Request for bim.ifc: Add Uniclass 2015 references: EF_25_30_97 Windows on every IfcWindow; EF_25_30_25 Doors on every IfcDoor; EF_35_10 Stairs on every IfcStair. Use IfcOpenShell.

First a look at what the model holds.

```python
import ifcopenshell

model = ifcopenshell.open("bim.ifc")
print(model.schema)
print("classifications:", [c.Name for c in model.by_type("IfcClassification")])
for ifc_class in ("IfcDoor", "IfcRoof", "IfcStair", "IfcWall", "IfcWindow"):
    print(ifc_class, len(model.by_type(ifc_class)))
```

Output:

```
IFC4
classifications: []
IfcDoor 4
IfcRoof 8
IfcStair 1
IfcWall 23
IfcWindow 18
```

```python
import ifcopenshell
import ifcopenshell.api.classification

model = ifcopenshell.open("bim.ifc")

system = ifcopenshell.api.classification.add_classification(model, classification="Uniclass 2015")

codes = {
    "IfcWindow": ("EF_25_30_97", "Windows"),
    "IfcDoor": ("EF_25_30_25", "Doors"),
    "IfcStair": ("EF_35_10", "Stairs"),
}
for ifc_class, (code, name) in codes.items():
    products = model.by_type(ifc_class)
    ifcopenshell.api.classification.add_reference(
        model, products=products, classification=system, identification=code, name=name
    )
    print(code, len(products))

model.write("bim_v2.ifc")
```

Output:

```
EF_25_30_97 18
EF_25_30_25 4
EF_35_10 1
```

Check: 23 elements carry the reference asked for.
